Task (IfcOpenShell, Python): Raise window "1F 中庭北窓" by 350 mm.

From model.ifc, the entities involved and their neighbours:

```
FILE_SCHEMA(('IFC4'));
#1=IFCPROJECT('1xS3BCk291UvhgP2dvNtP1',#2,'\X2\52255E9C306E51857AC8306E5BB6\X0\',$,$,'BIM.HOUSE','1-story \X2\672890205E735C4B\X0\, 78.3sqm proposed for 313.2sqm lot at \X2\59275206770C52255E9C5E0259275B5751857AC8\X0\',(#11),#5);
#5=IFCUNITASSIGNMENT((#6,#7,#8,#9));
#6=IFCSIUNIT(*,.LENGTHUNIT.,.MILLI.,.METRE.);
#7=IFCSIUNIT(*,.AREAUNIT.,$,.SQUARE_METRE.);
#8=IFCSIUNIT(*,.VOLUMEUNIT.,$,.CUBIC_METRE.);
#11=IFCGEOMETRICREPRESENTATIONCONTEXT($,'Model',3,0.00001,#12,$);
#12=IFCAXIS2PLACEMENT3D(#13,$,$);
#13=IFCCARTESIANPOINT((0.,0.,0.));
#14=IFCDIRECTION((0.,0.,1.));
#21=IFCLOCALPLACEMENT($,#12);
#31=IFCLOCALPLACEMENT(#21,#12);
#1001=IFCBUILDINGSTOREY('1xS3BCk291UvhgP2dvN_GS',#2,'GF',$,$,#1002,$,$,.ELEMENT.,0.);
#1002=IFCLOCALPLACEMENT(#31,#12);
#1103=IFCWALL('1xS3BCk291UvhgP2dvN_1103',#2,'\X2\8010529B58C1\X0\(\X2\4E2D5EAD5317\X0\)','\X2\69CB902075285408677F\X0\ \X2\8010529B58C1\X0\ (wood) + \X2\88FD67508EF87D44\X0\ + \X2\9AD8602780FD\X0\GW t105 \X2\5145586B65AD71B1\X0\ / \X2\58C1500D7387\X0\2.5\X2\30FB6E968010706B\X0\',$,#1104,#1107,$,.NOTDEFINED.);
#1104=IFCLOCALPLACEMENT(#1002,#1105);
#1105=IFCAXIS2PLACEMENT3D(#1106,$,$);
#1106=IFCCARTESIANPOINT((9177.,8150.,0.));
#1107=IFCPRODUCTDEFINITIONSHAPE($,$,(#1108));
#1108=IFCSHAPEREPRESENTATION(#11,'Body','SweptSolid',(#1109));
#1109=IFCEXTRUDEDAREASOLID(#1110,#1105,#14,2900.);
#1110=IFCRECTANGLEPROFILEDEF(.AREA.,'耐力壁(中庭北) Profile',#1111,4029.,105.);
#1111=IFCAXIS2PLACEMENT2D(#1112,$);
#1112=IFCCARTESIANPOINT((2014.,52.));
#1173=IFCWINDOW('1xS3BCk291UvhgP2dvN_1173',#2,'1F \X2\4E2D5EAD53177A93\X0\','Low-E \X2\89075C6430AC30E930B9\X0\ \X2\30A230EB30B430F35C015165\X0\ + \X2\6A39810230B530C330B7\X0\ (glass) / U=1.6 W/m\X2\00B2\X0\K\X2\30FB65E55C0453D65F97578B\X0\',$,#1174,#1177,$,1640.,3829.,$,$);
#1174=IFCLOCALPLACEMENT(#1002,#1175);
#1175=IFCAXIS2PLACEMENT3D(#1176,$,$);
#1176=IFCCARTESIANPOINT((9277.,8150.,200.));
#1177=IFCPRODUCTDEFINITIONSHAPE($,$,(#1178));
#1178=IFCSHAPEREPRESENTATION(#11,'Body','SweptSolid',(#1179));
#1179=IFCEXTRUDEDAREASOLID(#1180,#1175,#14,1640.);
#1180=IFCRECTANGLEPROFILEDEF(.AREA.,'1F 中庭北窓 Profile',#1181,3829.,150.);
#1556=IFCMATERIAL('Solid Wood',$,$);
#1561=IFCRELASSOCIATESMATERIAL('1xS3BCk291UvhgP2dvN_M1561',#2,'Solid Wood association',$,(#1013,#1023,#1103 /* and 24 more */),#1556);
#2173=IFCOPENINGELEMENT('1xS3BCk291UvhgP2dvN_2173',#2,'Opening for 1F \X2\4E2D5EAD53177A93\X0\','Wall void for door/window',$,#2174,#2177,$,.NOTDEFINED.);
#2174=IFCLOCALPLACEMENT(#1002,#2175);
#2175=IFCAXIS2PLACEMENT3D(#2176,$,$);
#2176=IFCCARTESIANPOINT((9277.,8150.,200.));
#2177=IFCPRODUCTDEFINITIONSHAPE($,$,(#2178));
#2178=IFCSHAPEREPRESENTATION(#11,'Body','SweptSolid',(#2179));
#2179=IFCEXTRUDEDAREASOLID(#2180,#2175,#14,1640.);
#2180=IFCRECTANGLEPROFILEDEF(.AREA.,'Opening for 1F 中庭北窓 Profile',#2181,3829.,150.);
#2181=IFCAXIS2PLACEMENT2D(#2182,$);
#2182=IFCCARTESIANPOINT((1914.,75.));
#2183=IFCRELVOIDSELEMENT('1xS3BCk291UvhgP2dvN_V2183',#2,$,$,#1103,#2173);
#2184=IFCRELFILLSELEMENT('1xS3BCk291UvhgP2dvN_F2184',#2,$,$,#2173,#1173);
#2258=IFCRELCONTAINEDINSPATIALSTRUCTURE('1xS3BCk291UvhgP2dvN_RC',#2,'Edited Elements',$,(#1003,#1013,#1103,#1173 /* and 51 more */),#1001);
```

```python
import numpy as np
import ifcopenshell
import ifcopenshell.api.geometry
import ifcopenshell.util.placement
import ifcopenshell.util.unit

model = ifcopenshell.open("model.ifc")
unit_scale = ifcopenshell.util.unit.calculate_unit_scale(model)

window = model.by_id(1173)
opening = window.FillsVoids[0].RelatingOpeningElement
dz = 0.35 / unit_scale

shift = np.array([0.0, 0.0, dz])
# The window is not placed relative to its opening, so move both.
for product in (opening, window):
    matrix = ifcopenshell.util.placement.get_local_placement(product.ObjectPlacement)
    matrix[:3, 3] += shift
    ifcopenshell.api.geometry.edit_object_placement(model, product=product, matrix=matrix, is_si=False)

print(f"moved by {dz * unit_scale:+.3f} m")

model.write("model_rev.ifc")
```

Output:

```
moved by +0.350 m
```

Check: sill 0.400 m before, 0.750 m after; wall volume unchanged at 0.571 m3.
